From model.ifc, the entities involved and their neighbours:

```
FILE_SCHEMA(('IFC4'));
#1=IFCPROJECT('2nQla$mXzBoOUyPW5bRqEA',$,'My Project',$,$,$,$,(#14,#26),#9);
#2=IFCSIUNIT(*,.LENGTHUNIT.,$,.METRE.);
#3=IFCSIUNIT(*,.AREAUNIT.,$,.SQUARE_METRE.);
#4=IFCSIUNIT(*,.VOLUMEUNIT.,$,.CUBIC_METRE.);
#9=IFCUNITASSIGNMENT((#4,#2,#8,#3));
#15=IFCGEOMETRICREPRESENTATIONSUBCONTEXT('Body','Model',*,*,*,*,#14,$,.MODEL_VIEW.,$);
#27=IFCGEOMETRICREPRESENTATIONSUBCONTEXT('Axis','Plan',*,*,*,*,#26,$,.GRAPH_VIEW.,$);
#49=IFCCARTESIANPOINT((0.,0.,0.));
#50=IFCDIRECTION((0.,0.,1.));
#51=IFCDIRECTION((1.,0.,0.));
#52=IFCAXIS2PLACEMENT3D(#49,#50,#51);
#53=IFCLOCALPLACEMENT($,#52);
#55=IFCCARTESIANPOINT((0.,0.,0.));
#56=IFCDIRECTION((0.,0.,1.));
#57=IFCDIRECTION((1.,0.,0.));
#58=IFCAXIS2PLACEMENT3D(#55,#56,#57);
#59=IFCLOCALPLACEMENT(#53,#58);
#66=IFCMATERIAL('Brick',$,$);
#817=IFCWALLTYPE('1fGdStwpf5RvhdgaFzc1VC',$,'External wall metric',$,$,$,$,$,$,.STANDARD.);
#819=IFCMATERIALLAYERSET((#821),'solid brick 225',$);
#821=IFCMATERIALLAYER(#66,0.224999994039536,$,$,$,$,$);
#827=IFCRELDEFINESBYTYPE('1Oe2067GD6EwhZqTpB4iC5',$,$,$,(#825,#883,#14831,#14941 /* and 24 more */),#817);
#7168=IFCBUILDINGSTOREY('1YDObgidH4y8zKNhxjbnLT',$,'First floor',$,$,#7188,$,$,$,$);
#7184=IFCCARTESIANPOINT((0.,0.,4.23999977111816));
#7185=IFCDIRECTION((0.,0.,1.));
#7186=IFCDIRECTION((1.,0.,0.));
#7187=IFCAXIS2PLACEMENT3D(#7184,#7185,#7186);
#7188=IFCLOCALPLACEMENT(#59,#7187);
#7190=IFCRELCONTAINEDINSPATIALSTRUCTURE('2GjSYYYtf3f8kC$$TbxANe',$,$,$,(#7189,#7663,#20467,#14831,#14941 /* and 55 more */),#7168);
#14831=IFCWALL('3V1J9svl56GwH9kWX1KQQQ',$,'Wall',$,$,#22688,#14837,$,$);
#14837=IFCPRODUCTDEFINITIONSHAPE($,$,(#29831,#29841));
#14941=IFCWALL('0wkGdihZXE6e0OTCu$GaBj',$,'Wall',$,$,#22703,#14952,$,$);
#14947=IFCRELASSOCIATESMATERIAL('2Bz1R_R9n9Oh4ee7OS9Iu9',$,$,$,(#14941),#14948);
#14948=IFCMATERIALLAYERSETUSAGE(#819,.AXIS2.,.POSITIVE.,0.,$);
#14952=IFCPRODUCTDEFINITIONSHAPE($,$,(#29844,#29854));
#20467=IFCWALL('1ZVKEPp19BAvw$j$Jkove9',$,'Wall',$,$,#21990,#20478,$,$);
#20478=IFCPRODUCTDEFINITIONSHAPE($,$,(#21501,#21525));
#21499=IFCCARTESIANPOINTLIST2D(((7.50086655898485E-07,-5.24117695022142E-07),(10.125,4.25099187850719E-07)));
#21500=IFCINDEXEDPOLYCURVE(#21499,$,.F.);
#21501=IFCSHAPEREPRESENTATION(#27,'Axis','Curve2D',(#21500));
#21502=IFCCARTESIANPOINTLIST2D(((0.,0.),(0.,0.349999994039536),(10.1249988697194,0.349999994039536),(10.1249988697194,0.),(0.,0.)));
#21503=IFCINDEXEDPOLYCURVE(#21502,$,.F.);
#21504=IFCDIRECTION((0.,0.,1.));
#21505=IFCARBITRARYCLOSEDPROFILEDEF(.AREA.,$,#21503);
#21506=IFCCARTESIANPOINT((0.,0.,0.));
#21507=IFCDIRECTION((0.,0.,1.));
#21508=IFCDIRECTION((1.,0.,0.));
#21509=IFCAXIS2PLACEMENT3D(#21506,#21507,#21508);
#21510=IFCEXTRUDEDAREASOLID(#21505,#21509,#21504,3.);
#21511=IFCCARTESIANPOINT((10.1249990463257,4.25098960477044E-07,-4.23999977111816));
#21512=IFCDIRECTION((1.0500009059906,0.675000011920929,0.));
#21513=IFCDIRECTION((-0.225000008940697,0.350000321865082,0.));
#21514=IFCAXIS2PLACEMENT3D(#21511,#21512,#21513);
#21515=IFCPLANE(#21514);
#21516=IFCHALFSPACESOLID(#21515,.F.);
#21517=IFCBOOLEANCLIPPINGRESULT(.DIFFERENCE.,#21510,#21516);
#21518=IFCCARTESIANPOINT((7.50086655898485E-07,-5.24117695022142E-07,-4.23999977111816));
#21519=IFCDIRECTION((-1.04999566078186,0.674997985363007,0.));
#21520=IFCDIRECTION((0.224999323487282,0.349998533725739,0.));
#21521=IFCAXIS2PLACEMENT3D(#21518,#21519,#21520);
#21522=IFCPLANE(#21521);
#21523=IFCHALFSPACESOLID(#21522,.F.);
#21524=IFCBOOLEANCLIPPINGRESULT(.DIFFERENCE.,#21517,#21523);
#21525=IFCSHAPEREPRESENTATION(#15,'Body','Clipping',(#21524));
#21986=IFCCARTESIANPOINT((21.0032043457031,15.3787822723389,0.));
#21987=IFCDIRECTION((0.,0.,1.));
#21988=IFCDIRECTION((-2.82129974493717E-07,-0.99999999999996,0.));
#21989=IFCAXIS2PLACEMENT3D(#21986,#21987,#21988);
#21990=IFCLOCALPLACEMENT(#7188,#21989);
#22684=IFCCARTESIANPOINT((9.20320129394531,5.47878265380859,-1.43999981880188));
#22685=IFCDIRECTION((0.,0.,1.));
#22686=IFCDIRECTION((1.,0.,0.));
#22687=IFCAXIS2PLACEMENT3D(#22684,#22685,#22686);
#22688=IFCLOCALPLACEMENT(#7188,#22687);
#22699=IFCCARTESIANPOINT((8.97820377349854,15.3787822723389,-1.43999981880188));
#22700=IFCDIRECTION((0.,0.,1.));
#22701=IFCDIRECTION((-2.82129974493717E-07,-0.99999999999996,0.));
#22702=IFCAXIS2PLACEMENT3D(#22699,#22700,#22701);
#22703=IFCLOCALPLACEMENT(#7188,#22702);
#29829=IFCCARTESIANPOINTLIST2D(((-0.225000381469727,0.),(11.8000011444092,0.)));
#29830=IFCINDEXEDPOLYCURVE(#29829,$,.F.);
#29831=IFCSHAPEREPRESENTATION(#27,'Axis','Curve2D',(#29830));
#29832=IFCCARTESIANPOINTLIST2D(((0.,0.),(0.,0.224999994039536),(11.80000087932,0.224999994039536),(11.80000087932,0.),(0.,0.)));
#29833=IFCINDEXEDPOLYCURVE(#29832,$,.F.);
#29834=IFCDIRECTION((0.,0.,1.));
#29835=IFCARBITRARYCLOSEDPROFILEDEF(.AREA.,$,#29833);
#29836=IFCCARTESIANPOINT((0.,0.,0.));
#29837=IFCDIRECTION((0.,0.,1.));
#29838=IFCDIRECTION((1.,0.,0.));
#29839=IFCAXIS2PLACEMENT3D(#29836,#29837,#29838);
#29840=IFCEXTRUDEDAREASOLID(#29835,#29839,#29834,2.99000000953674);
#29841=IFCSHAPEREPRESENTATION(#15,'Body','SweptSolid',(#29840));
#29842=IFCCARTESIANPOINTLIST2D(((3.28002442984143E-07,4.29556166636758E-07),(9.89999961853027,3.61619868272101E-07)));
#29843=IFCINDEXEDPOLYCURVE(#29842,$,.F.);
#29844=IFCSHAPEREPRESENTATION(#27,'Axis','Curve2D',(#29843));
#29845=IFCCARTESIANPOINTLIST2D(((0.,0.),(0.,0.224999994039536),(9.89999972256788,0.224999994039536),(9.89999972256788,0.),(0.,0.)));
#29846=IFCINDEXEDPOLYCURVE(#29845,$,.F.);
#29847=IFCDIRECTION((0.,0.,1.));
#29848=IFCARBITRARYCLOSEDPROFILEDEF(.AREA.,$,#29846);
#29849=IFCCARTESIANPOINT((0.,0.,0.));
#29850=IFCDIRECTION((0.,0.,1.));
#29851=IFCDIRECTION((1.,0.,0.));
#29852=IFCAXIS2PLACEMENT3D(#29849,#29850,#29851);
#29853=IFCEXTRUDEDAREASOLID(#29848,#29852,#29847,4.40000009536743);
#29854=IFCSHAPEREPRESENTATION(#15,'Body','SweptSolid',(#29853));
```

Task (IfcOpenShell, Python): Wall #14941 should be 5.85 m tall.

```python
import ifcopenshell
import ifcopenshell.geom
import ifcopenshell.util.representation
import ifcopenshell.util.shape
import ifcopenshell.util.unit

model = ifcopenshell.open("model.ifc")
unit_scale = ifcopenshell.util.unit.calculate_unit_scale(model)
settings = ifcopenshell.geom.settings()


def volume(element):
    """Net volume in cubic metres, openings subtracted."""
    shape = ifcopenshell.geom.create_shape(settings, element)
    return ifcopenshell.util.shape.get_volume(shape.geometry)


wall = model.by_id(14941)
before = volume(wall)

body = ifcopenshell.util.representation.get_representation(wall, "Model", "Body")
solid = body.Items[0]
old_height = solid.Depth
solid.Depth = 5.85 / unit_scale
after = volume(wall)

print(f"height {old_height:g} -> {solid.Depth:g}, volume {before:.3f} -> {after:.3f} m3")

model.write("model_v2.ifc")
```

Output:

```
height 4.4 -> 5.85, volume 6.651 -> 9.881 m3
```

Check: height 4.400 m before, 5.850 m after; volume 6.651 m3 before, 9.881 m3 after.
